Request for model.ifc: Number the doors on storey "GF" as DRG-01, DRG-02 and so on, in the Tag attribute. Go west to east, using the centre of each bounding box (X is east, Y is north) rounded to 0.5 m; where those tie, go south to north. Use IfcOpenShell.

First a look at what the model holds.

```python
import ifcopenshell
import ifcopenshell.util.element
import ifcopenshell.util.placement

model = ifcopenshell.open("model.ifc")
print(model.schema)
storey = next(s for s in model.by_type("IfcBuildingStorey") if s.Name == "GF")
doors = [e for e in ifcopenshell.util.element.get_decomposition(storey) if e.is_a("IfcDoor")]
for e in sorted(doors, key=lambda e: e.id()):
    origin = ifcopenshell.util.placement.get_local_placement(e.ObjectPlacement)[:3, 3]
    print(e.id(), e.Tag, e.Name, origin.round(2) + 0.0, sep=" | ")
```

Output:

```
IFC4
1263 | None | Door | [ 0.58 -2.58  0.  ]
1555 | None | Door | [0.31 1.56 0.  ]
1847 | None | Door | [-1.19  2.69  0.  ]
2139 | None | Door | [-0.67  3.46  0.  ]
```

```python
import ifcopenshell
import ifcopenshell.geom
import ifcopenshell.util.element
import ifcopenshell.util.shape

model = ifcopenshell.open("model.ifc")
settings = ifcopenshell.geom.settings()
settings.set("use-world-coords", True)


def centre(element):
    shape = ifcopenshell.geom.create_shape(settings, element)
    return ifcopenshell.util.shape.get_bbox_centroid(shape.geometry)


storey = next(s for s in model.by_type("IfcBuildingStorey") if s.Name == "GF")
doors = [e for e in ifcopenshell.util.element.get_decomposition(storey) if e.is_a("IfcDoor")]

# Insertion points can sit at a corner or the storey origin, so sort by the geometry (in metres).
centres = {e: centre(e) for e in doors}
doors.sort(key=lambda e: (round(centres[e][0] / 0.5), centres[e][1]))

for i, e in enumerate(doors, start=1):
    number = f"DRG-{i:02d}"
    e.Tag = number
    print(e.id(), number)

model.write("model_v2.ifc")
```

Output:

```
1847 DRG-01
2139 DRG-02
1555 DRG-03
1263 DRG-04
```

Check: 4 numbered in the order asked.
